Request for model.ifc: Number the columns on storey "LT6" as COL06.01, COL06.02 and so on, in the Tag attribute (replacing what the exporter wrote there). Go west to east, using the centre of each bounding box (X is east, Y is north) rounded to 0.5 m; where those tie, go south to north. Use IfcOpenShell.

First a look at what the model holds.

```python
import ifcopenshell
import ifcopenshell.util.element
import ifcopenshell.util.placement

model = ifcopenshell.open("model.ifc")
print(model.schema)
storey = next(s for s in model.by_type("IfcBuildingStorey") if s.Name == "LT6")
columns = [e for e in ifcopenshell.util.element.get_decomposition(storey) if e.is_a("IfcColumn")]
for e in sorted(columns, key=lambda e: e.id()):
    origin = ifcopenshell.util.placement.get_local_placement(e.ObjectPlacement)[:3, 3]
    print(e.id(), e.Tag, e.Name, origin.round(2) + 0.0, sep=" | ")
```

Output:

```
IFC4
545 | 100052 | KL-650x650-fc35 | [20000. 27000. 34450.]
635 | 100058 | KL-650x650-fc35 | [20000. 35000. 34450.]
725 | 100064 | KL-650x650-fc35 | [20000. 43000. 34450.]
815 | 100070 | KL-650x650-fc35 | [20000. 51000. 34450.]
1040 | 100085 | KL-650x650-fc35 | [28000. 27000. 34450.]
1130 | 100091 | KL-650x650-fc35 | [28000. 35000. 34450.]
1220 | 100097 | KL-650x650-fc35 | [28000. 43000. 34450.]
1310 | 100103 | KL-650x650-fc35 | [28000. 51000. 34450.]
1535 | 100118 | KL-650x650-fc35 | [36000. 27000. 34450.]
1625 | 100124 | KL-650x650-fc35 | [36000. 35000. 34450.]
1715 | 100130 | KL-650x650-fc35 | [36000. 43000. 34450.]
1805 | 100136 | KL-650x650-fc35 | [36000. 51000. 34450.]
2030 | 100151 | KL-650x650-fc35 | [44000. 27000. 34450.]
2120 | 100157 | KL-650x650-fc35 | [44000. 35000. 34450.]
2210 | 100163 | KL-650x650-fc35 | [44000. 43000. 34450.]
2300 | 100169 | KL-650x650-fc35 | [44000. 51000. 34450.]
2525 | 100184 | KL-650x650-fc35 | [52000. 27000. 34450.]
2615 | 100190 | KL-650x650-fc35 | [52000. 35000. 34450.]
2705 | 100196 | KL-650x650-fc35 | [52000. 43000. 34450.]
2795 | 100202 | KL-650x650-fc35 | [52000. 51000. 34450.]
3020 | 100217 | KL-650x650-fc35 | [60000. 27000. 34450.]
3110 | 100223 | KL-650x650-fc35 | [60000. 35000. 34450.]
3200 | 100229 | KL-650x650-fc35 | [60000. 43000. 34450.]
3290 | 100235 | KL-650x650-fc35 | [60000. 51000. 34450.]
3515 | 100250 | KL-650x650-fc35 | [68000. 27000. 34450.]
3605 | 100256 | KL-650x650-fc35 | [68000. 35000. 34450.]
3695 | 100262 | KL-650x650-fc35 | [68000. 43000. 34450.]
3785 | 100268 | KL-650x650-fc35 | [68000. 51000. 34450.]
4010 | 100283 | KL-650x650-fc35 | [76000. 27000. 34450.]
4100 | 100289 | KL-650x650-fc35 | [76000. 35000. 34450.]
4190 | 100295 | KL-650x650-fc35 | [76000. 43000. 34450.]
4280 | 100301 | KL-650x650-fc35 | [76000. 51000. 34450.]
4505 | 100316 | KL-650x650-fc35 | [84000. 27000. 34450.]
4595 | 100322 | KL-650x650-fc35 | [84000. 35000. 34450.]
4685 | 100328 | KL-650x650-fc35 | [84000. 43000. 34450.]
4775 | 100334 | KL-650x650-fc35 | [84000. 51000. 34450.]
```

```python
import ifcopenshell
import ifcopenshell.geom
import ifcopenshell.util.element
import ifcopenshell.util.shape

model = ifcopenshell.open("model.ifc")
settings = ifcopenshell.geom.settings()
settings.set("use-world-coords", True)


def centre(element):
    shape = ifcopenshell.geom.create_shape(settings, element)
    return ifcopenshell.util.shape.get_bbox_centroid(shape.geometry)


storey = next(s for s in model.by_type("IfcBuildingStorey") if s.Name == "LT6")
columns = [e for e in ifcopenshell.util.element.get_decomposition(storey) if e.is_a("IfcColumn")]

# Insertion points can sit at a corner or the storey origin, so sort by the geometry (in metres).
centres = {e: centre(e) for e in columns}
columns.sort(key=lambda e: (round(centres[e][0] / 0.5), centres[e][1]))

for i, e in enumerate(columns, start=1):
    number = f"COL06.{i:02d}"
    e.Tag = number
    print(e.id(), number)

model.write("model-out.ifc")
```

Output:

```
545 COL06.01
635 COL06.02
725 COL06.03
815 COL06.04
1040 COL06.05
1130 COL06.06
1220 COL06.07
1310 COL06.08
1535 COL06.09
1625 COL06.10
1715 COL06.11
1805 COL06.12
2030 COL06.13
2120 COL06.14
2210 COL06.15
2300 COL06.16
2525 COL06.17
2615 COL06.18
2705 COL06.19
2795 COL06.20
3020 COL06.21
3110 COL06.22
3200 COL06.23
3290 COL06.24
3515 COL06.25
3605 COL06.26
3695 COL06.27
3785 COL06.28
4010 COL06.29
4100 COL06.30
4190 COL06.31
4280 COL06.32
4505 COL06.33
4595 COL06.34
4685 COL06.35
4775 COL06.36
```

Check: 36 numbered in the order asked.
